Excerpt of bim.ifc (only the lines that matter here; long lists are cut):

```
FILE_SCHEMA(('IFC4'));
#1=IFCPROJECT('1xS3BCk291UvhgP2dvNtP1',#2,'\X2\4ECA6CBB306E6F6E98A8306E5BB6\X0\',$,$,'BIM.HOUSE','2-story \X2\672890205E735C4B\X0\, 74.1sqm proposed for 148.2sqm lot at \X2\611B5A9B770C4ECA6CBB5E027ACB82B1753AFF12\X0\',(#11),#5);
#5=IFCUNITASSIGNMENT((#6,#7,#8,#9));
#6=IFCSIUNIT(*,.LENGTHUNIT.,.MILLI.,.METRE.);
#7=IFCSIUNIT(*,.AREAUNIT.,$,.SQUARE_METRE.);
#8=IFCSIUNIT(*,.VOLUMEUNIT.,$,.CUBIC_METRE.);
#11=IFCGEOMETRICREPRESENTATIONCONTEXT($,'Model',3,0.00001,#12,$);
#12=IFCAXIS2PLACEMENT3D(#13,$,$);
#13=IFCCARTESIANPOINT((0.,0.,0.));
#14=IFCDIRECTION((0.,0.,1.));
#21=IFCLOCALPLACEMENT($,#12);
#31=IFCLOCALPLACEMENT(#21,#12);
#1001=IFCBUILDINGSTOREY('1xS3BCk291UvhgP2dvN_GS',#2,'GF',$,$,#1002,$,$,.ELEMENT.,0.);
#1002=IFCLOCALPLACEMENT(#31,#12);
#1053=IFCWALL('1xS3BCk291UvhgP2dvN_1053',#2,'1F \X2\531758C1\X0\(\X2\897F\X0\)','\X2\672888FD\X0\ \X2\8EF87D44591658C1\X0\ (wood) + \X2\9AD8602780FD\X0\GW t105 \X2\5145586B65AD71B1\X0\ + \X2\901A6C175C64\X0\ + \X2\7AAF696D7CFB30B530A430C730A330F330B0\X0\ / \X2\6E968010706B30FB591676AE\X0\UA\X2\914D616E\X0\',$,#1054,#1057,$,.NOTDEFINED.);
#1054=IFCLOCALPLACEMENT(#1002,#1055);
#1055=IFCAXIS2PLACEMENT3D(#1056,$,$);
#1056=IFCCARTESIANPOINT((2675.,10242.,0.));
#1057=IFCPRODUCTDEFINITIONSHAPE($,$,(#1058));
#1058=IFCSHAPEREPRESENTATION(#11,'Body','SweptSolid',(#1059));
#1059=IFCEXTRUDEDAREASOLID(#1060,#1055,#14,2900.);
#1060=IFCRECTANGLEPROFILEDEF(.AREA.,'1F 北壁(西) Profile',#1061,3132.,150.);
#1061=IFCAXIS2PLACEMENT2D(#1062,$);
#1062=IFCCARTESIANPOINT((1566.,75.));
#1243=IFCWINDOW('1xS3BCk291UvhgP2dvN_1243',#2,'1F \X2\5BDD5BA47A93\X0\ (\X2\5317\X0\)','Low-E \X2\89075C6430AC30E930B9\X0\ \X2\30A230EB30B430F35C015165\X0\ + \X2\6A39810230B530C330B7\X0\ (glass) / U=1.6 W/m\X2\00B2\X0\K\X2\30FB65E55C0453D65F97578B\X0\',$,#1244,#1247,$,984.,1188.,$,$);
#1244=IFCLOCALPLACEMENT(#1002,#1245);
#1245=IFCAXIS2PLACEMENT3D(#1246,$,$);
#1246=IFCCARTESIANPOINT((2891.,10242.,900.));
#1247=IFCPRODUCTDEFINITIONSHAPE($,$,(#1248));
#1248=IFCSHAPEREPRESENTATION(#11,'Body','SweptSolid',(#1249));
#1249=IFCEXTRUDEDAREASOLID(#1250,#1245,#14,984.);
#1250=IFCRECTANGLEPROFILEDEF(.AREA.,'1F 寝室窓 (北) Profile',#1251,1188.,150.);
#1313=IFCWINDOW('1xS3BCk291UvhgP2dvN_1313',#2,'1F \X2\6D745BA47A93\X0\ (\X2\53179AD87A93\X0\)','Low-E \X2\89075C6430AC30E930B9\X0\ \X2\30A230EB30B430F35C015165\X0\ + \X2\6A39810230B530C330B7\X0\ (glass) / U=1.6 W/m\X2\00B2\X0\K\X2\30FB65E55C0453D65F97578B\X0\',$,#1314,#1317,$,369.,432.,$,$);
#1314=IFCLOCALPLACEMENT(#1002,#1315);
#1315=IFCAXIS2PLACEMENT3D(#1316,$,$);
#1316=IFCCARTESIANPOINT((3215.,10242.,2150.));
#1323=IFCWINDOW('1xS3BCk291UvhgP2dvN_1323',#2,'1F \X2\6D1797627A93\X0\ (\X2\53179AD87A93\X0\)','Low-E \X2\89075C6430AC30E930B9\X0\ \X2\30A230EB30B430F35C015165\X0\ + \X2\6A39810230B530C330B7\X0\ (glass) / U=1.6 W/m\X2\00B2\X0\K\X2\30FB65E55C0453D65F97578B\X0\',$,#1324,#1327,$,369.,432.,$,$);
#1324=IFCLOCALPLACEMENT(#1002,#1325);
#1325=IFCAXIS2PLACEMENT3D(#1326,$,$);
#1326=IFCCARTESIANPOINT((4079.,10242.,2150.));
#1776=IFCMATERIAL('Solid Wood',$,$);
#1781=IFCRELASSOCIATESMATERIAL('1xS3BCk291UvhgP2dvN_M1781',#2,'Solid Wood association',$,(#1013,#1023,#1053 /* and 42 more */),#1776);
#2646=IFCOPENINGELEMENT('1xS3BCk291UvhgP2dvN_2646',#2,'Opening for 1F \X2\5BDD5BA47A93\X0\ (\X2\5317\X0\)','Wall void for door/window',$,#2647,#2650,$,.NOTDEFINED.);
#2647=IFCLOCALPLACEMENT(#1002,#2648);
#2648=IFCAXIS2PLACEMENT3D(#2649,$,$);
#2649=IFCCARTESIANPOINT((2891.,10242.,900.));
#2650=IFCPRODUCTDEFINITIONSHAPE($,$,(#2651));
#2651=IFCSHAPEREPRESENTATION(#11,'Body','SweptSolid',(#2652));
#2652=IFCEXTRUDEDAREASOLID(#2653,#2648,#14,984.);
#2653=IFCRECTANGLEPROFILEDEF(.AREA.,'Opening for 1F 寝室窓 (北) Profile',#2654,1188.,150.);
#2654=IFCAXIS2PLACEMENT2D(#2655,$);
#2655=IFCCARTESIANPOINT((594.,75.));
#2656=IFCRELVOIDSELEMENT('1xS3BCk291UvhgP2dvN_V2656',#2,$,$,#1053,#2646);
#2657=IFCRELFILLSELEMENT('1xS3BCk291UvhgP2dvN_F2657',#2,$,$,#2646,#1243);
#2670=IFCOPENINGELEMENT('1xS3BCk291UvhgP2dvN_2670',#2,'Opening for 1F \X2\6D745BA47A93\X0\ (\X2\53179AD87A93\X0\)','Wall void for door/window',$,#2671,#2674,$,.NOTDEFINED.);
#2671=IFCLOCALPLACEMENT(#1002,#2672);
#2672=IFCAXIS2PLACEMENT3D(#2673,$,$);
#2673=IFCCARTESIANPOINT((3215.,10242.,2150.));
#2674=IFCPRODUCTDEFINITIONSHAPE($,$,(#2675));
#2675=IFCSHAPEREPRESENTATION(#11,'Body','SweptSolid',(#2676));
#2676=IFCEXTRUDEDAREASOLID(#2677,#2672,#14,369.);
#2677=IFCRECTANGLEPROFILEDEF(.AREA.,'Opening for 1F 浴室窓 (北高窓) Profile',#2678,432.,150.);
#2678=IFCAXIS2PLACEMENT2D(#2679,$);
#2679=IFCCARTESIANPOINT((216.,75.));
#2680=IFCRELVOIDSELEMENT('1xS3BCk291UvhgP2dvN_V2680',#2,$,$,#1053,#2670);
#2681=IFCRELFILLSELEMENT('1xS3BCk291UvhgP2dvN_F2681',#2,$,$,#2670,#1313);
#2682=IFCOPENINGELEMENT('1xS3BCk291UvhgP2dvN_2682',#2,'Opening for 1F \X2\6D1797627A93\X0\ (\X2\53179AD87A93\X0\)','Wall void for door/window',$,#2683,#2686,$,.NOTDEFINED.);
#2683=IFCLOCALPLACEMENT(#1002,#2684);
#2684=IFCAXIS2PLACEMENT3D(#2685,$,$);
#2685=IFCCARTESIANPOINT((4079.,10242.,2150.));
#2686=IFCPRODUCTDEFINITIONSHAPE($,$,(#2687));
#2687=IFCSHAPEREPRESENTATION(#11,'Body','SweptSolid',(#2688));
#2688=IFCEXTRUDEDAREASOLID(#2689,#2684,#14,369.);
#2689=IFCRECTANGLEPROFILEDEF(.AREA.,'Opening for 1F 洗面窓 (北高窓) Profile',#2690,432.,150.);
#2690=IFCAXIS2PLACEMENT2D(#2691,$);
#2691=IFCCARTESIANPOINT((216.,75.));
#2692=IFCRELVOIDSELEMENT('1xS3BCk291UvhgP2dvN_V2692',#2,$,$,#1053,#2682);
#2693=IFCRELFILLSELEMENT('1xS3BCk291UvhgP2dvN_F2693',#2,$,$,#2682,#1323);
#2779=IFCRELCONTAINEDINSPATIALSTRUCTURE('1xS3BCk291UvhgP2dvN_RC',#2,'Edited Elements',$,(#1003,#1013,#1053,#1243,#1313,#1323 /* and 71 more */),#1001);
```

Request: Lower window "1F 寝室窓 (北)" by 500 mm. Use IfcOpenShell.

```python
import numpy as np
import ifcopenshell
import ifcopenshell.api.geometry
import ifcopenshell.util.placement
import ifcopenshell.util.unit

model = ifcopenshell.open("bim.ifc")
unit_scale = ifcopenshell.util.unit.calculate_unit_scale(model)

window = model.by_guid("1xS3BCk291UvhgP2dvN_1243")
opening = window.FillsVoids[0].RelatingOpeningElement
dz = -500.0

shift = np.array([0.0, 0.0, dz])
# The window is not placed relative to its opening, so move both.
for product in (opening, window):
    matrix = ifcopenshell.util.placement.get_local_placement(product.ObjectPlacement)
    matrix[:3, 3] += shift
    ifcopenshell.api.geometry.edit_object_placement(model, product=product, matrix=matrix, is_si=False)

print(f"moved by {dz * unit_scale:+.3f} m")

model.write("bim_rev.ifc")
```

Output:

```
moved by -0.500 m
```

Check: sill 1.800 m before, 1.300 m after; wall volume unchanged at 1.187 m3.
